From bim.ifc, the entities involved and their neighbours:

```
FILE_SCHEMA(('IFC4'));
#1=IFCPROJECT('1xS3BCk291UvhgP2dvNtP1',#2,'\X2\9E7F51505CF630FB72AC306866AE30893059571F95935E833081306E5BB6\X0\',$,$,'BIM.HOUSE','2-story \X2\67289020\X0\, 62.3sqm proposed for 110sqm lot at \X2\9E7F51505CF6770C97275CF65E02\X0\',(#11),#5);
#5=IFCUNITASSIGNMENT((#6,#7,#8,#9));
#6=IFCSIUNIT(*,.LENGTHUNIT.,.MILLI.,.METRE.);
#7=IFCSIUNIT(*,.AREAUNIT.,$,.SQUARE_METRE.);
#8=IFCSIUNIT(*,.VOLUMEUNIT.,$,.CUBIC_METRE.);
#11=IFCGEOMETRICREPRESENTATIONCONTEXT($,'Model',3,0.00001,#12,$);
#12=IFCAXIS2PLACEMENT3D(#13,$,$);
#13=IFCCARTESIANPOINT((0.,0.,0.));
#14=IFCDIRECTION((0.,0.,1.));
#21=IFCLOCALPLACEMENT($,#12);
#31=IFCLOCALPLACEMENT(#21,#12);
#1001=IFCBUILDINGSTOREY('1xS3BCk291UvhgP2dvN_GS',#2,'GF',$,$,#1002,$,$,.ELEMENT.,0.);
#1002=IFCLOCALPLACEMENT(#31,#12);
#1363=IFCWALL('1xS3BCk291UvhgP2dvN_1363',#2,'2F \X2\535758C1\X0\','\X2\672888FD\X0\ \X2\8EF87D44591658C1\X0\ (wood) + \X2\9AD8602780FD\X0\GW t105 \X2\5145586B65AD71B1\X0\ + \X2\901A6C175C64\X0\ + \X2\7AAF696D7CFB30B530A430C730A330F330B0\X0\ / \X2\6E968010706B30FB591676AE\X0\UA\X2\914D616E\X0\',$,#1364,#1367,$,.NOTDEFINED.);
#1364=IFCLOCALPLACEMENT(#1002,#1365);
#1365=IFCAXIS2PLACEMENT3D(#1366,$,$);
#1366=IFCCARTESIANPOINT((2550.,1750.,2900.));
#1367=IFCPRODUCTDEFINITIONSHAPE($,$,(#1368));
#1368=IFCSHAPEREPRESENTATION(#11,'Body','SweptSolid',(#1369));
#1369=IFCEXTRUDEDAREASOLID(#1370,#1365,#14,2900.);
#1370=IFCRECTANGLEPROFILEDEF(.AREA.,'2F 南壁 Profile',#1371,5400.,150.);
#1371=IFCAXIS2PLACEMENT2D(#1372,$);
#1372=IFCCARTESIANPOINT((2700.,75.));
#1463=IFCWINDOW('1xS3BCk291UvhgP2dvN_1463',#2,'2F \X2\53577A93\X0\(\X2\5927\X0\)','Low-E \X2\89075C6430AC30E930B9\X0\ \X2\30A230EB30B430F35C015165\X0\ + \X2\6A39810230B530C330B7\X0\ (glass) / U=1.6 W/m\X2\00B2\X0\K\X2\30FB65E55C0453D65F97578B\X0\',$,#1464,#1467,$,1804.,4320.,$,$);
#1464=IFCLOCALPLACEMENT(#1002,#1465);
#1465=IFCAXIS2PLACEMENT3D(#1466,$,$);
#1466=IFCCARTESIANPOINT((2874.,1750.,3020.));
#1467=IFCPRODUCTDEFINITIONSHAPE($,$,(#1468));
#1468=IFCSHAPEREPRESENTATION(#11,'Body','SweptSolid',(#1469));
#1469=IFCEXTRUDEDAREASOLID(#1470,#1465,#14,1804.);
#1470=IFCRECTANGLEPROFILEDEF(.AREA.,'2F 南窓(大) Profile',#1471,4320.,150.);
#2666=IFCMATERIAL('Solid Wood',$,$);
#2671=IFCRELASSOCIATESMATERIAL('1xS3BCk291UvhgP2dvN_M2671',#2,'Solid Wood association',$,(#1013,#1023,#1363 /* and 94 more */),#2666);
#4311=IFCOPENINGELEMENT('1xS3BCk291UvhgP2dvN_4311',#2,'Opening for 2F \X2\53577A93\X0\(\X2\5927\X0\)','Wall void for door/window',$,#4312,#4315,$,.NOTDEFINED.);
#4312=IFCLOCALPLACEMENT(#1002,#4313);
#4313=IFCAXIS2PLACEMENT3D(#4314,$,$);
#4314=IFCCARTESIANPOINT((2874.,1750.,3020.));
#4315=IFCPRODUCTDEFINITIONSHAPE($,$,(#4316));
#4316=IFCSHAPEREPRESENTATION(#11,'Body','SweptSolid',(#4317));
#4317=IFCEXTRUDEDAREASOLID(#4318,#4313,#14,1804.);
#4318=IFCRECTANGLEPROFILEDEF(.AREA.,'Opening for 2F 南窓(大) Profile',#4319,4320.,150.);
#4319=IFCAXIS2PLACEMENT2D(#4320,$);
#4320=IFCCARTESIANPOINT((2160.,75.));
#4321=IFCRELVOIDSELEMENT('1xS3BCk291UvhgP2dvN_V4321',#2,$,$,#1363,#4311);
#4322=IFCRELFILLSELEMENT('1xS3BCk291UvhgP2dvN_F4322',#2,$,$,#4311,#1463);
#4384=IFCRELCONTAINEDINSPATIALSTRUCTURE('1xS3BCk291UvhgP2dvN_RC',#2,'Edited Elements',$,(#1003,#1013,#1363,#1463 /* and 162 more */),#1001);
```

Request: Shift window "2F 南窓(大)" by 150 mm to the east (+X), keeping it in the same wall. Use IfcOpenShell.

```python
import ifcopenshell
import ifcopenshell.api.geometry
import ifcopenshell.util.placement
import ifcopenshell.util.unit

model = ifcopenshell.open("bim.ifc")
unit_scale = ifcopenshell.util.unit.calculate_unit_scale(model)

window = model.by_guid("1xS3BCk291UvhgP2dvN_1463")
opening = window.FillsVoids[0].RelatingOpeningElement
wall = opening.VoidsElements[0].RelatingBuildingElement

wall_matrix = ifcopenshell.util.placement.get_local_placement(wall.ObjectPlacement)
shift = wall_matrix[:3, 0] * 0.15 / unit_scale
before = ifcopenshell.util.placement.get_local_placement(window.ObjectPlacement)[:3, 3].copy()

# The window is not placed relative to its opening, so move both.
for product in (opening, window):
    matrix = ifcopenshell.util.placement.get_local_placement(product.ObjectPlacement)
    matrix[:3, 3] += shift
    ifcopenshell.api.geometry.edit_object_placement(model, product=product, matrix=matrix, is_si=False)

after = ifcopenshell.util.placement.get_local_placement(window.ObjectPlacement)[:3, 3]
print("window moved by", (after - before).round(3) + 0.0)

model.write("bim_edited.ifc")
```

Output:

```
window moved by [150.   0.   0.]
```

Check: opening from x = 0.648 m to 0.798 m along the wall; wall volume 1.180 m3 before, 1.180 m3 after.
